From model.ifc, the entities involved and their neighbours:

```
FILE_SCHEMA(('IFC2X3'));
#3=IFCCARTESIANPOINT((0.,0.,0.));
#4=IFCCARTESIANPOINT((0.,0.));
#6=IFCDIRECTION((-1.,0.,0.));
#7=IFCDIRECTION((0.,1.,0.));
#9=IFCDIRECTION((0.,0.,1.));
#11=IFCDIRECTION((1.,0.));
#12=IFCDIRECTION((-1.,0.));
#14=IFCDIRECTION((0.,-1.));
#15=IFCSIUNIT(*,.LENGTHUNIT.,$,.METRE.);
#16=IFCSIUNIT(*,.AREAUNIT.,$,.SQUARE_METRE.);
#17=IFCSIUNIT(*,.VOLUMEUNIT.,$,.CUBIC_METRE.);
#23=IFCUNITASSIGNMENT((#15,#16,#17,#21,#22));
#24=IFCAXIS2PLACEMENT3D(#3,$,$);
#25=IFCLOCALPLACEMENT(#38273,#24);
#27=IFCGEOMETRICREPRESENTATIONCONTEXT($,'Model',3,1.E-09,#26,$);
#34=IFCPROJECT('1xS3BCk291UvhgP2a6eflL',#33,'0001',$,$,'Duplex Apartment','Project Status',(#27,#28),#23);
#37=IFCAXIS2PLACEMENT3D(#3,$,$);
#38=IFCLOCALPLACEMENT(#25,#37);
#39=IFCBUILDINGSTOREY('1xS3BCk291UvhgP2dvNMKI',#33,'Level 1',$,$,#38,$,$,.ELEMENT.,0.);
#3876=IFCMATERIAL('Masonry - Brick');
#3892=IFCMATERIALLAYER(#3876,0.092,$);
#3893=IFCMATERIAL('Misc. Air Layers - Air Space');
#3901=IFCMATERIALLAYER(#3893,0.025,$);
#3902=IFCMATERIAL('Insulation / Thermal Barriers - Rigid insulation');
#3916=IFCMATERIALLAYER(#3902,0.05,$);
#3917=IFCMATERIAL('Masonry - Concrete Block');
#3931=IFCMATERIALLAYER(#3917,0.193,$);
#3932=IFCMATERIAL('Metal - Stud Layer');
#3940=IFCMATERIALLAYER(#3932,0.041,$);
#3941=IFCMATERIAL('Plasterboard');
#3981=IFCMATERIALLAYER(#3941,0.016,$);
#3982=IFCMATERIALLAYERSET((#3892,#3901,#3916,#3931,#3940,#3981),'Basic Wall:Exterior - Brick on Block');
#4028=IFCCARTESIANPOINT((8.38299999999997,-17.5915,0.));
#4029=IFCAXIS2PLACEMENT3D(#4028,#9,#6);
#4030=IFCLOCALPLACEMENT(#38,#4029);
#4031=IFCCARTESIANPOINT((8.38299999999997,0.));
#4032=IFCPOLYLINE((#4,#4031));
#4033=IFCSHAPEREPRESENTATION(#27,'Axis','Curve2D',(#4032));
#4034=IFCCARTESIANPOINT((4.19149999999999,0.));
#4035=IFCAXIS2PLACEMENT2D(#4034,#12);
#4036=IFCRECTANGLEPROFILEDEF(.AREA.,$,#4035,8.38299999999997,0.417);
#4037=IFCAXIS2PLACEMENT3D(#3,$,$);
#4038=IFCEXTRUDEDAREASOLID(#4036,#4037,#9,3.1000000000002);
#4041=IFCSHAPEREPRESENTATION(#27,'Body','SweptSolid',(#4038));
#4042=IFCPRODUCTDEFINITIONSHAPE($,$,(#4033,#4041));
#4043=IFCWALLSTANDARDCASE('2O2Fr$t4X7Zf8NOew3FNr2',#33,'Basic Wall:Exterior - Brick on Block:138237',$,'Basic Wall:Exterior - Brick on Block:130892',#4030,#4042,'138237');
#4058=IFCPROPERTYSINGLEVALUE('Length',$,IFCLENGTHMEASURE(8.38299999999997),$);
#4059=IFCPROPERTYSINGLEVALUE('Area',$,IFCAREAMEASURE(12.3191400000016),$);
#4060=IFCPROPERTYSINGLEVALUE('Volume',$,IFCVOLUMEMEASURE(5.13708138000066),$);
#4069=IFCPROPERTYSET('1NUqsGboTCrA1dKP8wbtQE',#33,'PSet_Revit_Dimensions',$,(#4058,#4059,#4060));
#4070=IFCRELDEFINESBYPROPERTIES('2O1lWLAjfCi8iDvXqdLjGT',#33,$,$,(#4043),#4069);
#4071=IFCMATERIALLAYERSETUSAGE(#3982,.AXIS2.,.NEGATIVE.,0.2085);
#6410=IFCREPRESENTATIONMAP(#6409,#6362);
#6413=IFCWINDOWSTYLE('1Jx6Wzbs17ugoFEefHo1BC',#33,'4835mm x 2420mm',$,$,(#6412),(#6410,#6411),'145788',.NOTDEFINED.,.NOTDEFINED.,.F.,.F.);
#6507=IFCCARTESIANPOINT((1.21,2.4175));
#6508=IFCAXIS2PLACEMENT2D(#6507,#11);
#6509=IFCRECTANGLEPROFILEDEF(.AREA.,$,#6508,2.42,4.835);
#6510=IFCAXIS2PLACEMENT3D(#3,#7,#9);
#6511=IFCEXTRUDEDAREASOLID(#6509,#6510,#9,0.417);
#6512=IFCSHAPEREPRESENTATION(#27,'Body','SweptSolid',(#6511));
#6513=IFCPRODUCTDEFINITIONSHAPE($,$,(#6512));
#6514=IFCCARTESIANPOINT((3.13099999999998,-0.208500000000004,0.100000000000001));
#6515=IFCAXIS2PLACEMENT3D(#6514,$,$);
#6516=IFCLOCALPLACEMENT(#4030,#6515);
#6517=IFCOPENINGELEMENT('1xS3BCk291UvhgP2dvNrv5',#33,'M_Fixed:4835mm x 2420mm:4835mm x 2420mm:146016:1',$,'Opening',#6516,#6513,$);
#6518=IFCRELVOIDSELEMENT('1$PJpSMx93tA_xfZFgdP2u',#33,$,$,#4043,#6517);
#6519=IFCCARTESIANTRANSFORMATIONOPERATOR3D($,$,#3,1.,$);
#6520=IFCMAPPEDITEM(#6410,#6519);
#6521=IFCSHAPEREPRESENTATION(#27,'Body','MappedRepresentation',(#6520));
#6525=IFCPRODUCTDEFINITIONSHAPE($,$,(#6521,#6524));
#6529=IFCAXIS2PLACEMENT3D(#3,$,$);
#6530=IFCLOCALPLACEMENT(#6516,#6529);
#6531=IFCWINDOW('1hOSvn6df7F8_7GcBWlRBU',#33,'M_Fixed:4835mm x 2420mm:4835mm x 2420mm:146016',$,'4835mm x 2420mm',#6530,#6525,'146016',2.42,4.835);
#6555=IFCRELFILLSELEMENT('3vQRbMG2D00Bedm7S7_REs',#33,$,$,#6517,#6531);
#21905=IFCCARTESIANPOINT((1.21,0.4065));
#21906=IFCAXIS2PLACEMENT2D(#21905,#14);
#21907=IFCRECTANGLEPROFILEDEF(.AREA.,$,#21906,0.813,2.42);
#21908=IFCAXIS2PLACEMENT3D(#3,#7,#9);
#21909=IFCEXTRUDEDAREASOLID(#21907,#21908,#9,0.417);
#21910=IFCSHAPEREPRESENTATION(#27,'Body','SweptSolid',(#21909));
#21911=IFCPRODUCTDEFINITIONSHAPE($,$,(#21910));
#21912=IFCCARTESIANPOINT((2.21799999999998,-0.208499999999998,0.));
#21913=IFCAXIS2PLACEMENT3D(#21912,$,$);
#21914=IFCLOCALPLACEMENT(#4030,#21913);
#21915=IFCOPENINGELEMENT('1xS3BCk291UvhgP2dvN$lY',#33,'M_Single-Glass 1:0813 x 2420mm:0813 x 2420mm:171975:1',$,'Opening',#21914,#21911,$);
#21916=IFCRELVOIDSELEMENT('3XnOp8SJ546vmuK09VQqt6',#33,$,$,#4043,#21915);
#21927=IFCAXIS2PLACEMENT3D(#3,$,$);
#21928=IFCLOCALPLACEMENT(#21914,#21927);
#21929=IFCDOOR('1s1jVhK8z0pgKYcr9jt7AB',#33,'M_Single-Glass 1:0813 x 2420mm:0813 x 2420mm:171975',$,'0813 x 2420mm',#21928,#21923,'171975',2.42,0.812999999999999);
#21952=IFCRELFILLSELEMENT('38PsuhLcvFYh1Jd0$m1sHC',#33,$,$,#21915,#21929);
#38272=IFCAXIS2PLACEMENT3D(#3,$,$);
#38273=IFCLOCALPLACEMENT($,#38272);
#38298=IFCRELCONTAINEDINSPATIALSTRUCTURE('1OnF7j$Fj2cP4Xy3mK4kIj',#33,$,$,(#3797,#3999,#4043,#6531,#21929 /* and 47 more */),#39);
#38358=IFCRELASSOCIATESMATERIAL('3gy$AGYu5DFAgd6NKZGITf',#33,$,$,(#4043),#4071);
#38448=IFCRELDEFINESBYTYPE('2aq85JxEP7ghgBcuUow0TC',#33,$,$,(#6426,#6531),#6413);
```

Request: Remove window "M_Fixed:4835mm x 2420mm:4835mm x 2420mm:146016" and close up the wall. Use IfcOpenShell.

```python
import ifcopenshell
import ifcopenshell.api.feature
import ifcopenshell.api.pset
import ifcopenshell.api.root
import ifcopenshell.geom
import ifcopenshell.util.element
import ifcopenshell.util.shape
import ifcopenshell.util.unit

model = ifcopenshell.open("model.ifc")
area_scale = ifcopenshell.util.unit.calculate_unit_scale(model, "AREAUNIT")
volume_scale = ifcopenshell.util.unit.calculate_unit_scale(model, "VOLUMEUNIT")
settings = ifcopenshell.geom.settings()


def volume(element):
    """Net volume in cubic metres, openings subtracted."""
    shape = ifcopenshell.geom.create_shape(settings, element)
    return ifcopenshell.util.shape.get_volume(shape.geometry)


window = model.by_guid("1hOSvn6df7F8_7GcBWlRBU")
opening = window.FillsVoids[0].RelatingOpeningElement
wall = opening.VoidsElements[0].RelatingBuildingElement
before = volume(wall)

ifcopenshell.api.root.remove_product(model, product=window)
ifcopenshell.api.feature.remove_feature(model, feature=opening)

after = volume(wall)
thickness = 0.417  # wall thickness in metres

# Update the wall's stored quantities.
pset = model.by_id(ifcopenshell.util.element.get_pset(wall, "PSet_Revit_Dimensions", should_inherit=False)["id"])
ifcopenshell.api.pset.edit_pset(model, pset=pset, properties={
    "Area": model.create_entity("IfcAreaMeasure", after / thickness / area_scale),
    "Volume": model.create_entity("IfcVolumeMeasure", after / volume_scale),
})

print(f"wall volume {before:.3f} -> {after:.3f} m3")

model.write("model_v2.ifc")
```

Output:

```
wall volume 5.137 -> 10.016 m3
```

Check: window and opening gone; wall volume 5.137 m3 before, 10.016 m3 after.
